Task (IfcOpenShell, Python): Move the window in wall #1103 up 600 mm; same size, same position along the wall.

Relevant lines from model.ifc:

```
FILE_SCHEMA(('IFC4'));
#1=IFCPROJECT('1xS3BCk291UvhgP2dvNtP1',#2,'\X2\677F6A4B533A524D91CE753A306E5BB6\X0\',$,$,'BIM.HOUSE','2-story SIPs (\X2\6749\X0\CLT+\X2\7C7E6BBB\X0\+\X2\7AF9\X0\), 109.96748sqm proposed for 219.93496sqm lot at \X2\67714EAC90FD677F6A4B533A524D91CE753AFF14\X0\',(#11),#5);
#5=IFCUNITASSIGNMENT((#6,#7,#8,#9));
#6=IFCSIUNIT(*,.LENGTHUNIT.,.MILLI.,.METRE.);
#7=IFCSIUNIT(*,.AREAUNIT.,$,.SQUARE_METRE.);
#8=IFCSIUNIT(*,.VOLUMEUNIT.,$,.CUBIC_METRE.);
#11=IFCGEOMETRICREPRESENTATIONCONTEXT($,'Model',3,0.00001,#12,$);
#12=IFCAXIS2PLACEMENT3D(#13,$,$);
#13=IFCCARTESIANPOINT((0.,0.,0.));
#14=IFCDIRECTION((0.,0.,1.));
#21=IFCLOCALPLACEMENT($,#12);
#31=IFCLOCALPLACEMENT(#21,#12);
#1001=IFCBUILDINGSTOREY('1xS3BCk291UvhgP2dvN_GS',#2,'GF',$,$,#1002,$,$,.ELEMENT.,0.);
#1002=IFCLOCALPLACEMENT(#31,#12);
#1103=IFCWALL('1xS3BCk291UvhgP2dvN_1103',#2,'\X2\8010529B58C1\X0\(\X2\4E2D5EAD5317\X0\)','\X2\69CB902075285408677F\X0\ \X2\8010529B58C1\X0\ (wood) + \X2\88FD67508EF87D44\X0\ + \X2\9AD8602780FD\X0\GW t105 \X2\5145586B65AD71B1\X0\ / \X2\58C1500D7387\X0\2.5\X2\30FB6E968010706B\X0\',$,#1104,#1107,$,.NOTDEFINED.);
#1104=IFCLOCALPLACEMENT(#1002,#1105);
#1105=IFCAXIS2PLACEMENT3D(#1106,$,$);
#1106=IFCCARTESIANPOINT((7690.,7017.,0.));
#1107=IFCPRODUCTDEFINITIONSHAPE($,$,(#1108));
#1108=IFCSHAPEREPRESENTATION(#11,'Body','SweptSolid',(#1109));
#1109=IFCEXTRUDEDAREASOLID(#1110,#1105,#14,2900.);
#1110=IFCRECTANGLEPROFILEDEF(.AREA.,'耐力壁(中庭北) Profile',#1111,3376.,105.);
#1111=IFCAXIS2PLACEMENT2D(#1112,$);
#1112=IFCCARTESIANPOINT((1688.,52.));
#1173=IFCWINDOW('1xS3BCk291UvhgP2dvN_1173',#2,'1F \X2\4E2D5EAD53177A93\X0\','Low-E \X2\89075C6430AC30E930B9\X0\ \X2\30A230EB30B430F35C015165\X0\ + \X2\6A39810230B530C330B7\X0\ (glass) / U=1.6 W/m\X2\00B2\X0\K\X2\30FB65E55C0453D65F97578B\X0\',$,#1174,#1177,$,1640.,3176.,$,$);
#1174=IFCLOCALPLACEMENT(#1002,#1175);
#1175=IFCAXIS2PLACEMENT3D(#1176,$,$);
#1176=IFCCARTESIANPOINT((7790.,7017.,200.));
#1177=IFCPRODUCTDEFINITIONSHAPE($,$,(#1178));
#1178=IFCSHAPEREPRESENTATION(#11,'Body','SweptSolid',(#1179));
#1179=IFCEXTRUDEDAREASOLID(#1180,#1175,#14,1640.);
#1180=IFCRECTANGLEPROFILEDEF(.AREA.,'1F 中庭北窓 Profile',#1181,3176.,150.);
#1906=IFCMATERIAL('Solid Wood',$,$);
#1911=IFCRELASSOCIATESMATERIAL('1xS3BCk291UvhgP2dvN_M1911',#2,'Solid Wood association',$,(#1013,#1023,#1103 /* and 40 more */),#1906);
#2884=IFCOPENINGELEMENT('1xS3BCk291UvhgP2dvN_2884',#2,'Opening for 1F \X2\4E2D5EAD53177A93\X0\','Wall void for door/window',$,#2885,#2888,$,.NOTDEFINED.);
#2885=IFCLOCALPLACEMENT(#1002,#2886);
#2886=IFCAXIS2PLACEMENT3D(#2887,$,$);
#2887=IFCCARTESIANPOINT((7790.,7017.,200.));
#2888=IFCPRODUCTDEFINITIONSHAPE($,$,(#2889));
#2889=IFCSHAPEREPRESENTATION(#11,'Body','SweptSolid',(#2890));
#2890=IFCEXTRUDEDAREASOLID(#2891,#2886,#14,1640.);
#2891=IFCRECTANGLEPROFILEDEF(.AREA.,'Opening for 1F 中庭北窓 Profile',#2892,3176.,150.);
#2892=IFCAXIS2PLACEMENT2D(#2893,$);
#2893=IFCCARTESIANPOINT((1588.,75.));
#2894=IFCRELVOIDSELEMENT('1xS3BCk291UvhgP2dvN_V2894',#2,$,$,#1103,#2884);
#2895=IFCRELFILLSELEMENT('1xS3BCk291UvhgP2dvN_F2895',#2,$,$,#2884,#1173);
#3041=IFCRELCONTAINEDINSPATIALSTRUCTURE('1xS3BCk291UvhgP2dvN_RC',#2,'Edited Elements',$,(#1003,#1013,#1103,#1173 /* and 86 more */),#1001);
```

```python
import numpy as np
import ifcopenshell
import ifcopenshell.api.geometry
import ifcopenshell.util.placement
import ifcopenshell.util.unit

model = ifcopenshell.open("model.ifc")
unit_scale = ifcopenshell.util.unit.calculate_unit_scale(model)

window = model.by_guid("1xS3BCk291UvhgP2dvN_1173")
opening = window.FillsVoids[0].RelatingOpeningElement
dz = 600.0

shift = np.array([0.0, 0.0, dz])
# The window is not placed relative to its opening, so move both.
for product in (opening, window):
    matrix = ifcopenshell.util.placement.get_local_placement(product.ObjectPlacement)
    matrix[:3, 3] += shift
    ifcopenshell.api.geometry.edit_object_placement(model, product=product, matrix=matrix, is_si=False)

print(f"moved by {dz * unit_scale:+.3f} m")

model.write("model_rev.ifc")
```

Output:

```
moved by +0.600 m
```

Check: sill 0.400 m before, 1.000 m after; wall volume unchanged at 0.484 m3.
